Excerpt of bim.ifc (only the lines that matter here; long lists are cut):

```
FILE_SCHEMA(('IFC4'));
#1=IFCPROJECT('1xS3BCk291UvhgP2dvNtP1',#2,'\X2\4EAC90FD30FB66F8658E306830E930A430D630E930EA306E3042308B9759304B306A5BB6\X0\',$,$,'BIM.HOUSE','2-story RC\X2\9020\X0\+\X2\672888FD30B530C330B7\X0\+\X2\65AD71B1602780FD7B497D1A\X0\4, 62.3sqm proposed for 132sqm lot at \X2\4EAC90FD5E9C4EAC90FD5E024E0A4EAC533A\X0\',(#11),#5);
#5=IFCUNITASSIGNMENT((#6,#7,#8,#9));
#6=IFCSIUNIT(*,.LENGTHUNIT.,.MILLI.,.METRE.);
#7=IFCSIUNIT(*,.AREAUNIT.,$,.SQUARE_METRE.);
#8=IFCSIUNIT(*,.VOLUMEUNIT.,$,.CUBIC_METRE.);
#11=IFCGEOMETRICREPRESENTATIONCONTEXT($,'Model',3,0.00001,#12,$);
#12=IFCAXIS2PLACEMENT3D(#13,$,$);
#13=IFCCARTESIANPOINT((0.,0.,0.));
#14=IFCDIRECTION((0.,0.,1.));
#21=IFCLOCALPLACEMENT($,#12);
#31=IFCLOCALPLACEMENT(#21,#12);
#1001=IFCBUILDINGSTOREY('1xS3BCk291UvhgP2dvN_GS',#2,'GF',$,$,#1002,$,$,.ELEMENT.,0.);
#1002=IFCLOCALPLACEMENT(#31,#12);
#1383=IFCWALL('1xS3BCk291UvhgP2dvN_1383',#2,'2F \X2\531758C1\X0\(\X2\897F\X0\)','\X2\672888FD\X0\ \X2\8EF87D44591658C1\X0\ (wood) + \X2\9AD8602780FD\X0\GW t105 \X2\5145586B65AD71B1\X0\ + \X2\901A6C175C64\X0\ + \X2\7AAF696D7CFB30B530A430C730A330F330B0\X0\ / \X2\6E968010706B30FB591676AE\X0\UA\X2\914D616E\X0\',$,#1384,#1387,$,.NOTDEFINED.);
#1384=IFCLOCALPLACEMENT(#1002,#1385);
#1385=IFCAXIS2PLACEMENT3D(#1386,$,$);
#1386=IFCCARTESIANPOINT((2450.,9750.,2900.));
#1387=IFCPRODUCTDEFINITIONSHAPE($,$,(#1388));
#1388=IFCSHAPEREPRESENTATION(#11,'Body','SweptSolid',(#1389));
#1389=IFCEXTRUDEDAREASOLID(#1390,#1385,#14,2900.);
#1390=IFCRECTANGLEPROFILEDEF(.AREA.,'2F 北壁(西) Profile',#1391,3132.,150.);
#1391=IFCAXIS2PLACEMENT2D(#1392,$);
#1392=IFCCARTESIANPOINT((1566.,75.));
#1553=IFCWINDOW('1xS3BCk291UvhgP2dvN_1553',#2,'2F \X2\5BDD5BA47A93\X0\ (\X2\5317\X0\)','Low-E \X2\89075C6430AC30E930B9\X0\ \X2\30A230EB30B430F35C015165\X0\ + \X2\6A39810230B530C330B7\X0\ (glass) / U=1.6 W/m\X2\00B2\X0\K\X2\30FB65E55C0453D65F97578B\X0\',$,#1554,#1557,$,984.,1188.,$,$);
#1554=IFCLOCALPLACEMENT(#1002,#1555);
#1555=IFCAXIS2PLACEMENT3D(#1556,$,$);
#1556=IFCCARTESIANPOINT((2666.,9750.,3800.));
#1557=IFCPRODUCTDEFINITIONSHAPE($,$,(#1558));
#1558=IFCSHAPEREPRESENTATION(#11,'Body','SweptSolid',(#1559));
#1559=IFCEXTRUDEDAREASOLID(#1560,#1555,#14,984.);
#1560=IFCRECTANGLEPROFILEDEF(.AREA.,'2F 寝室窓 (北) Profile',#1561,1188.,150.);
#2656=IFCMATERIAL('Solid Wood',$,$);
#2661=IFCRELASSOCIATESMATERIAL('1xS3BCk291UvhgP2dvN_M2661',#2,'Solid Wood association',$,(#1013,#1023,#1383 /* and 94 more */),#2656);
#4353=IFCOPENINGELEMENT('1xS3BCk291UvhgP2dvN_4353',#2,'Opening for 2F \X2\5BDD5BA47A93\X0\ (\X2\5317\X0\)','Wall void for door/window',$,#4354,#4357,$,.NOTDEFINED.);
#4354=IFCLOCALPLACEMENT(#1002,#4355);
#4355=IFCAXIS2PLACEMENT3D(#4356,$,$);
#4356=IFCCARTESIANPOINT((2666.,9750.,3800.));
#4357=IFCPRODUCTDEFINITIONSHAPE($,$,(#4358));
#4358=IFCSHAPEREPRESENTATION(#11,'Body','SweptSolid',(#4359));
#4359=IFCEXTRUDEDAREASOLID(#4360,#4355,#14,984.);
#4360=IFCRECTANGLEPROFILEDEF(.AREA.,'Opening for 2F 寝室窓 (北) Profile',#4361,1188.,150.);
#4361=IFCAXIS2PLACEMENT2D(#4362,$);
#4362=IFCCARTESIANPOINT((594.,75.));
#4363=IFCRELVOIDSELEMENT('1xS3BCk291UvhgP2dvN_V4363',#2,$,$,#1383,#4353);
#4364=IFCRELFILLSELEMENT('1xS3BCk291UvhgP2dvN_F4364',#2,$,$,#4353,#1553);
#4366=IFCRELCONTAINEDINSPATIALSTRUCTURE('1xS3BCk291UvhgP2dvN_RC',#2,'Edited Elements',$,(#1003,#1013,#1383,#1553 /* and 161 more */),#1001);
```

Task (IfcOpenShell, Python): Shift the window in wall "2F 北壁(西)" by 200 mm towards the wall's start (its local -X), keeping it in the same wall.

```python
import ifcopenshell
import ifcopenshell.api.geometry
import ifcopenshell.util.placement

model = ifcopenshell.open("bim.ifc")

window = model.by_guid("1xS3BCk291UvhgP2dvN_1553")
opening = window.FillsVoids[0].RelatingOpeningElement
wall = opening.VoidsElements[0].RelatingBuildingElement

wall_matrix = ifcopenshell.util.placement.get_local_placement(wall.ObjectPlacement)
shift = wall_matrix[:3, 0] * -200.0
before = ifcopenshell.util.placement.get_local_placement(window.ObjectPlacement)[:3, 3].copy()

# The window is not placed relative to its opening, so move both.
for product in (opening, window):
    matrix = ifcopenshell.util.placement.get_local_placement(product.ObjectPlacement)
    matrix[:3, 3] += shift
    ifcopenshell.api.geometry.edit_object_placement(model, product=product, matrix=matrix, is_si=False)

after = ifcopenshell.util.placement.get_local_placement(window.ObjectPlacement)[:3, 3]
print("window moved by", (after - before).round(3) + 0.0)

model.write("bim_edited.ifc")
```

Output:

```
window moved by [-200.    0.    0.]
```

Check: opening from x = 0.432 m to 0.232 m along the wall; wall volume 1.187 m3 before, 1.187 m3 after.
